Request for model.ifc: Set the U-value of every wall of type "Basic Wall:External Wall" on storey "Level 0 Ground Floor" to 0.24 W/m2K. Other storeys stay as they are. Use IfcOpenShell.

First a look at what the model holds.

```python
import ifcopenshell
import ifcopenshell.util.element

model = ifcopenshell.open("model.ifc")
print(model.schema)
storey = next(s for s in model.by_type("IfcBuildingStorey") if s.Name == "Level 0 Ground Floor")
walls = [e for e in ifcopenshell.util.element.get_decomposition(storey) if e.is_a("IfcWall")]
seen = {}
for e in walls:
    element_type = ifcopenshell.util.element.get_type(e)
    key = (element_type.Name if element_type != e and element_type else None, ifcopenshell.util.element.get_pset(e, "Pset_WallCommon", "ThermalTransmittance"))
    seen[key] = seen.get(key, 0) + 1
for (name, value), count in sorted(seen.items(), key=str):
    print(count, "x", name, "|", value)
```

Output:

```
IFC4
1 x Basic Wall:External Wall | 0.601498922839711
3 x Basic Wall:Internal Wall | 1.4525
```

```python
import ifcopenshell
import ifcopenshell.api.pset
import ifcopenshell.util.element

model = ifcopenshell.open("model.ifc")

storey = next(s for s in model.by_type("IfcBuildingStorey") if s.Name == "Level 0 Ground Floor")
walls = [e for e in ifcopenshell.util.element.get_decomposition(storey) if e.is_a("IfcWall")]

count = 0
for e in walls:
    element_type = ifcopenshell.util.element.get_type(e)
    if element_type in (None, e) or element_type.Name != "Basic Wall:External Wall":
        continue
    # add_pset returns the element's existing set when there is one.
    pset = ifcopenshell.api.pset.add_pset(model, product=e, name="Pset_WallCommon")
    ifcopenshell.api.pset.edit_pset(model, pset=pset, properties={"ThermalTransmittance": 0.24})
    count += 1

print(count, "walls updated")

model.write("model_rev.ifc")
```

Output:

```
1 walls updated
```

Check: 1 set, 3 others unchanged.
